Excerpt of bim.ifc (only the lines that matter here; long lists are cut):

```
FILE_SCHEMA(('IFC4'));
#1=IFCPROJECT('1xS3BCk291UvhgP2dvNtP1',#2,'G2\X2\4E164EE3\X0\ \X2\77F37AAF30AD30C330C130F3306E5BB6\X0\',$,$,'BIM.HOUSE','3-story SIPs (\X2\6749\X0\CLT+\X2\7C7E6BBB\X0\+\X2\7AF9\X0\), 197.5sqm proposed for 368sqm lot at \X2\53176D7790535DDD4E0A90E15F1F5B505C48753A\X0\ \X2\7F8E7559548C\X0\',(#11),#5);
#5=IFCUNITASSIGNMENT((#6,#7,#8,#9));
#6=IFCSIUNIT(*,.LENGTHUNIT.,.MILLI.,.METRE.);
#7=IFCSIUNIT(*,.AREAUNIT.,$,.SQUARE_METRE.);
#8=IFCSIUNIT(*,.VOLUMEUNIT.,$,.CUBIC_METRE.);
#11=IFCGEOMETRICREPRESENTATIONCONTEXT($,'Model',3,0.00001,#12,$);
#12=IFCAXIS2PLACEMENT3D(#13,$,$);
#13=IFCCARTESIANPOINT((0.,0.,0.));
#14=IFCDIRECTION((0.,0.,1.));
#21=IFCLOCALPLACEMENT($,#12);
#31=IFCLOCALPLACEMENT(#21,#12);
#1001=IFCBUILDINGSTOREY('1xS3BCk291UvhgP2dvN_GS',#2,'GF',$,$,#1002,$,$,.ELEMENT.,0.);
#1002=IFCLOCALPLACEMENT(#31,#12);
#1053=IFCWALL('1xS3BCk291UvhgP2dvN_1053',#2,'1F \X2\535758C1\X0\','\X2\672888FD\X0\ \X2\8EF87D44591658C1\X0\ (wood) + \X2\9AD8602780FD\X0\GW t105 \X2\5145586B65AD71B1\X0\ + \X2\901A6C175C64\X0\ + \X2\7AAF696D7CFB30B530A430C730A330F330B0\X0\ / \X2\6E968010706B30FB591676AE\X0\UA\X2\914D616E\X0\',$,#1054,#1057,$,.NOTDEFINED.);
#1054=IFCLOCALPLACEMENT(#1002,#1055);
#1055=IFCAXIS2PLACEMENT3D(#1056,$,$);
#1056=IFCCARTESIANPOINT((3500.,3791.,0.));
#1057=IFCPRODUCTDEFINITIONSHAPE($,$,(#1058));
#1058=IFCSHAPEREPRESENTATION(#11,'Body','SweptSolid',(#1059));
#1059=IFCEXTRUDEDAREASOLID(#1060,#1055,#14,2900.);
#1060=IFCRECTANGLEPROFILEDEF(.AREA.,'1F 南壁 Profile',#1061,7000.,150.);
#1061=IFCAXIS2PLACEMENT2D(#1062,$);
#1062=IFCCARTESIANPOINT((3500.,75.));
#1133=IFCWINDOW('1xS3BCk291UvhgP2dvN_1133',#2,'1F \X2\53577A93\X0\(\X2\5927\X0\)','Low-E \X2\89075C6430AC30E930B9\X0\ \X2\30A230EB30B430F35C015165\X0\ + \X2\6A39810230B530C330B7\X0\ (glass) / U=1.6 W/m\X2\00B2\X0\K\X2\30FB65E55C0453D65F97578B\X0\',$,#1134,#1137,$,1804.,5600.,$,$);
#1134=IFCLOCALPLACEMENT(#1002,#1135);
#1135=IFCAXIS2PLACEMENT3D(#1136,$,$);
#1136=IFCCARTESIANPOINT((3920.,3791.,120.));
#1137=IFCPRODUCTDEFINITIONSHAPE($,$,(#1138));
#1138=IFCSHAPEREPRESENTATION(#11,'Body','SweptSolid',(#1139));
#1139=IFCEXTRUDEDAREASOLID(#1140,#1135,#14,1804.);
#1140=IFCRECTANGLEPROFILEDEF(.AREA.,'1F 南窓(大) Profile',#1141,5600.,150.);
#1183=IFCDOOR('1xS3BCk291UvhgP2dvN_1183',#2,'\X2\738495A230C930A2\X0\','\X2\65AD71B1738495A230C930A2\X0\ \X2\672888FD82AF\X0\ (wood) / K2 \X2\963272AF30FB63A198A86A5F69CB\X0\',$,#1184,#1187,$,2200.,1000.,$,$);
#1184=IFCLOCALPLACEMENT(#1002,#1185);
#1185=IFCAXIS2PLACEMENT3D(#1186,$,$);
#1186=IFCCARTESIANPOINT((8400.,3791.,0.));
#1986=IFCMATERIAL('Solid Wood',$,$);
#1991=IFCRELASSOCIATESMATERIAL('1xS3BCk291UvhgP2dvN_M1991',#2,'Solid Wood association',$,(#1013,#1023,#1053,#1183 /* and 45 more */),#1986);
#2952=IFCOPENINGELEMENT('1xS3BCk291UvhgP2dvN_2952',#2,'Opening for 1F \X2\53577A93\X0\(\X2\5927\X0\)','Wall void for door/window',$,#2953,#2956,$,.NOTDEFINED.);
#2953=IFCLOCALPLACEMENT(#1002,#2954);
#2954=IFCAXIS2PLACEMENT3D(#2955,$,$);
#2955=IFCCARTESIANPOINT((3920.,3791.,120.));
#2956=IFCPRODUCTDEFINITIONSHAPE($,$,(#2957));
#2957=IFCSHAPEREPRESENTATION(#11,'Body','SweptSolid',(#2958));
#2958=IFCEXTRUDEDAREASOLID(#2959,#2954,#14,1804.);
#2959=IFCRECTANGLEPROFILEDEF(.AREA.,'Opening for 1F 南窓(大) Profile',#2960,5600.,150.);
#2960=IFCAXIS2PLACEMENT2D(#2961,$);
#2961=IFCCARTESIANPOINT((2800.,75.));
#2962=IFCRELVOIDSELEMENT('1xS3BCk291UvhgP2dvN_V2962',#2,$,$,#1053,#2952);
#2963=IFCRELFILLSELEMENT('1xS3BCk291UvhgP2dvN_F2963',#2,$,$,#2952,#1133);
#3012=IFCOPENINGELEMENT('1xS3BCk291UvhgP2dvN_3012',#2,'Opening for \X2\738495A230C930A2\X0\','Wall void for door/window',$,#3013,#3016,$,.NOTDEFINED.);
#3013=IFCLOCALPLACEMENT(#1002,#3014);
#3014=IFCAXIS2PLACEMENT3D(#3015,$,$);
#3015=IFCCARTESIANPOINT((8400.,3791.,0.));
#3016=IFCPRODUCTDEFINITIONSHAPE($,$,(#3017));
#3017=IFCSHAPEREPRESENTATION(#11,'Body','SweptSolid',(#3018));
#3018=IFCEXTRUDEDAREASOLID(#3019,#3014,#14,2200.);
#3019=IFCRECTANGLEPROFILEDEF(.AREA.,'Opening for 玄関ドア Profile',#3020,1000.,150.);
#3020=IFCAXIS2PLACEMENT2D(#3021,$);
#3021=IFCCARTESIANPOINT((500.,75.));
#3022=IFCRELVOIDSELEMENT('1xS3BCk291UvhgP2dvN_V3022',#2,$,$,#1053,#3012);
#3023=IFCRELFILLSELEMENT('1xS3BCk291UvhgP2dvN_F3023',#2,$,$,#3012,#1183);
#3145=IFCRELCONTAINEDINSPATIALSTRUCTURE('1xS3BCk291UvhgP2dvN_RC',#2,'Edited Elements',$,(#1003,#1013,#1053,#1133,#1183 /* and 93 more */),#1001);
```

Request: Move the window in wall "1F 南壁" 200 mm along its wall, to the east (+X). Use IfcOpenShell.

```python
import ifcopenshell
import ifcopenshell.api.geometry
import ifcopenshell.util.placement
import ifcopenshell.util.unit

model = ifcopenshell.open("bim.ifc")
unit_scale = ifcopenshell.util.unit.calculate_unit_scale(model)

window = model.by_id(1133)
opening = window.FillsVoids[0].RelatingOpeningElement
wall = opening.VoidsElements[0].RelatingBuildingElement

wall_matrix = ifcopenshell.util.placement.get_local_placement(wall.ObjectPlacement)
shift = wall_matrix[:3, 0] * 0.2 / unit_scale
before = ifcopenshell.util.placement.get_local_placement(window.ObjectPlacement)[:3, 3].copy()

# The window is not placed relative to its opening, so move both.
for product in (opening, window):
    matrix = ifcopenshell.util.placement.get_local_placement(product.ObjectPlacement)
    matrix[:3, 3] += shift
    ifcopenshell.api.geometry.edit_object_placement(model, product=product, matrix=matrix, is_si=False)

after = ifcopenshell.util.placement.get_local_placement(window.ObjectPlacement)[:3, 3]
print("window moved by", (after - before).round(3) + 0.0)

model.write("bim_rev.ifc")
```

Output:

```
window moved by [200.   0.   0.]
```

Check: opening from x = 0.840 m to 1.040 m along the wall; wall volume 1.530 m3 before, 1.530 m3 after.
